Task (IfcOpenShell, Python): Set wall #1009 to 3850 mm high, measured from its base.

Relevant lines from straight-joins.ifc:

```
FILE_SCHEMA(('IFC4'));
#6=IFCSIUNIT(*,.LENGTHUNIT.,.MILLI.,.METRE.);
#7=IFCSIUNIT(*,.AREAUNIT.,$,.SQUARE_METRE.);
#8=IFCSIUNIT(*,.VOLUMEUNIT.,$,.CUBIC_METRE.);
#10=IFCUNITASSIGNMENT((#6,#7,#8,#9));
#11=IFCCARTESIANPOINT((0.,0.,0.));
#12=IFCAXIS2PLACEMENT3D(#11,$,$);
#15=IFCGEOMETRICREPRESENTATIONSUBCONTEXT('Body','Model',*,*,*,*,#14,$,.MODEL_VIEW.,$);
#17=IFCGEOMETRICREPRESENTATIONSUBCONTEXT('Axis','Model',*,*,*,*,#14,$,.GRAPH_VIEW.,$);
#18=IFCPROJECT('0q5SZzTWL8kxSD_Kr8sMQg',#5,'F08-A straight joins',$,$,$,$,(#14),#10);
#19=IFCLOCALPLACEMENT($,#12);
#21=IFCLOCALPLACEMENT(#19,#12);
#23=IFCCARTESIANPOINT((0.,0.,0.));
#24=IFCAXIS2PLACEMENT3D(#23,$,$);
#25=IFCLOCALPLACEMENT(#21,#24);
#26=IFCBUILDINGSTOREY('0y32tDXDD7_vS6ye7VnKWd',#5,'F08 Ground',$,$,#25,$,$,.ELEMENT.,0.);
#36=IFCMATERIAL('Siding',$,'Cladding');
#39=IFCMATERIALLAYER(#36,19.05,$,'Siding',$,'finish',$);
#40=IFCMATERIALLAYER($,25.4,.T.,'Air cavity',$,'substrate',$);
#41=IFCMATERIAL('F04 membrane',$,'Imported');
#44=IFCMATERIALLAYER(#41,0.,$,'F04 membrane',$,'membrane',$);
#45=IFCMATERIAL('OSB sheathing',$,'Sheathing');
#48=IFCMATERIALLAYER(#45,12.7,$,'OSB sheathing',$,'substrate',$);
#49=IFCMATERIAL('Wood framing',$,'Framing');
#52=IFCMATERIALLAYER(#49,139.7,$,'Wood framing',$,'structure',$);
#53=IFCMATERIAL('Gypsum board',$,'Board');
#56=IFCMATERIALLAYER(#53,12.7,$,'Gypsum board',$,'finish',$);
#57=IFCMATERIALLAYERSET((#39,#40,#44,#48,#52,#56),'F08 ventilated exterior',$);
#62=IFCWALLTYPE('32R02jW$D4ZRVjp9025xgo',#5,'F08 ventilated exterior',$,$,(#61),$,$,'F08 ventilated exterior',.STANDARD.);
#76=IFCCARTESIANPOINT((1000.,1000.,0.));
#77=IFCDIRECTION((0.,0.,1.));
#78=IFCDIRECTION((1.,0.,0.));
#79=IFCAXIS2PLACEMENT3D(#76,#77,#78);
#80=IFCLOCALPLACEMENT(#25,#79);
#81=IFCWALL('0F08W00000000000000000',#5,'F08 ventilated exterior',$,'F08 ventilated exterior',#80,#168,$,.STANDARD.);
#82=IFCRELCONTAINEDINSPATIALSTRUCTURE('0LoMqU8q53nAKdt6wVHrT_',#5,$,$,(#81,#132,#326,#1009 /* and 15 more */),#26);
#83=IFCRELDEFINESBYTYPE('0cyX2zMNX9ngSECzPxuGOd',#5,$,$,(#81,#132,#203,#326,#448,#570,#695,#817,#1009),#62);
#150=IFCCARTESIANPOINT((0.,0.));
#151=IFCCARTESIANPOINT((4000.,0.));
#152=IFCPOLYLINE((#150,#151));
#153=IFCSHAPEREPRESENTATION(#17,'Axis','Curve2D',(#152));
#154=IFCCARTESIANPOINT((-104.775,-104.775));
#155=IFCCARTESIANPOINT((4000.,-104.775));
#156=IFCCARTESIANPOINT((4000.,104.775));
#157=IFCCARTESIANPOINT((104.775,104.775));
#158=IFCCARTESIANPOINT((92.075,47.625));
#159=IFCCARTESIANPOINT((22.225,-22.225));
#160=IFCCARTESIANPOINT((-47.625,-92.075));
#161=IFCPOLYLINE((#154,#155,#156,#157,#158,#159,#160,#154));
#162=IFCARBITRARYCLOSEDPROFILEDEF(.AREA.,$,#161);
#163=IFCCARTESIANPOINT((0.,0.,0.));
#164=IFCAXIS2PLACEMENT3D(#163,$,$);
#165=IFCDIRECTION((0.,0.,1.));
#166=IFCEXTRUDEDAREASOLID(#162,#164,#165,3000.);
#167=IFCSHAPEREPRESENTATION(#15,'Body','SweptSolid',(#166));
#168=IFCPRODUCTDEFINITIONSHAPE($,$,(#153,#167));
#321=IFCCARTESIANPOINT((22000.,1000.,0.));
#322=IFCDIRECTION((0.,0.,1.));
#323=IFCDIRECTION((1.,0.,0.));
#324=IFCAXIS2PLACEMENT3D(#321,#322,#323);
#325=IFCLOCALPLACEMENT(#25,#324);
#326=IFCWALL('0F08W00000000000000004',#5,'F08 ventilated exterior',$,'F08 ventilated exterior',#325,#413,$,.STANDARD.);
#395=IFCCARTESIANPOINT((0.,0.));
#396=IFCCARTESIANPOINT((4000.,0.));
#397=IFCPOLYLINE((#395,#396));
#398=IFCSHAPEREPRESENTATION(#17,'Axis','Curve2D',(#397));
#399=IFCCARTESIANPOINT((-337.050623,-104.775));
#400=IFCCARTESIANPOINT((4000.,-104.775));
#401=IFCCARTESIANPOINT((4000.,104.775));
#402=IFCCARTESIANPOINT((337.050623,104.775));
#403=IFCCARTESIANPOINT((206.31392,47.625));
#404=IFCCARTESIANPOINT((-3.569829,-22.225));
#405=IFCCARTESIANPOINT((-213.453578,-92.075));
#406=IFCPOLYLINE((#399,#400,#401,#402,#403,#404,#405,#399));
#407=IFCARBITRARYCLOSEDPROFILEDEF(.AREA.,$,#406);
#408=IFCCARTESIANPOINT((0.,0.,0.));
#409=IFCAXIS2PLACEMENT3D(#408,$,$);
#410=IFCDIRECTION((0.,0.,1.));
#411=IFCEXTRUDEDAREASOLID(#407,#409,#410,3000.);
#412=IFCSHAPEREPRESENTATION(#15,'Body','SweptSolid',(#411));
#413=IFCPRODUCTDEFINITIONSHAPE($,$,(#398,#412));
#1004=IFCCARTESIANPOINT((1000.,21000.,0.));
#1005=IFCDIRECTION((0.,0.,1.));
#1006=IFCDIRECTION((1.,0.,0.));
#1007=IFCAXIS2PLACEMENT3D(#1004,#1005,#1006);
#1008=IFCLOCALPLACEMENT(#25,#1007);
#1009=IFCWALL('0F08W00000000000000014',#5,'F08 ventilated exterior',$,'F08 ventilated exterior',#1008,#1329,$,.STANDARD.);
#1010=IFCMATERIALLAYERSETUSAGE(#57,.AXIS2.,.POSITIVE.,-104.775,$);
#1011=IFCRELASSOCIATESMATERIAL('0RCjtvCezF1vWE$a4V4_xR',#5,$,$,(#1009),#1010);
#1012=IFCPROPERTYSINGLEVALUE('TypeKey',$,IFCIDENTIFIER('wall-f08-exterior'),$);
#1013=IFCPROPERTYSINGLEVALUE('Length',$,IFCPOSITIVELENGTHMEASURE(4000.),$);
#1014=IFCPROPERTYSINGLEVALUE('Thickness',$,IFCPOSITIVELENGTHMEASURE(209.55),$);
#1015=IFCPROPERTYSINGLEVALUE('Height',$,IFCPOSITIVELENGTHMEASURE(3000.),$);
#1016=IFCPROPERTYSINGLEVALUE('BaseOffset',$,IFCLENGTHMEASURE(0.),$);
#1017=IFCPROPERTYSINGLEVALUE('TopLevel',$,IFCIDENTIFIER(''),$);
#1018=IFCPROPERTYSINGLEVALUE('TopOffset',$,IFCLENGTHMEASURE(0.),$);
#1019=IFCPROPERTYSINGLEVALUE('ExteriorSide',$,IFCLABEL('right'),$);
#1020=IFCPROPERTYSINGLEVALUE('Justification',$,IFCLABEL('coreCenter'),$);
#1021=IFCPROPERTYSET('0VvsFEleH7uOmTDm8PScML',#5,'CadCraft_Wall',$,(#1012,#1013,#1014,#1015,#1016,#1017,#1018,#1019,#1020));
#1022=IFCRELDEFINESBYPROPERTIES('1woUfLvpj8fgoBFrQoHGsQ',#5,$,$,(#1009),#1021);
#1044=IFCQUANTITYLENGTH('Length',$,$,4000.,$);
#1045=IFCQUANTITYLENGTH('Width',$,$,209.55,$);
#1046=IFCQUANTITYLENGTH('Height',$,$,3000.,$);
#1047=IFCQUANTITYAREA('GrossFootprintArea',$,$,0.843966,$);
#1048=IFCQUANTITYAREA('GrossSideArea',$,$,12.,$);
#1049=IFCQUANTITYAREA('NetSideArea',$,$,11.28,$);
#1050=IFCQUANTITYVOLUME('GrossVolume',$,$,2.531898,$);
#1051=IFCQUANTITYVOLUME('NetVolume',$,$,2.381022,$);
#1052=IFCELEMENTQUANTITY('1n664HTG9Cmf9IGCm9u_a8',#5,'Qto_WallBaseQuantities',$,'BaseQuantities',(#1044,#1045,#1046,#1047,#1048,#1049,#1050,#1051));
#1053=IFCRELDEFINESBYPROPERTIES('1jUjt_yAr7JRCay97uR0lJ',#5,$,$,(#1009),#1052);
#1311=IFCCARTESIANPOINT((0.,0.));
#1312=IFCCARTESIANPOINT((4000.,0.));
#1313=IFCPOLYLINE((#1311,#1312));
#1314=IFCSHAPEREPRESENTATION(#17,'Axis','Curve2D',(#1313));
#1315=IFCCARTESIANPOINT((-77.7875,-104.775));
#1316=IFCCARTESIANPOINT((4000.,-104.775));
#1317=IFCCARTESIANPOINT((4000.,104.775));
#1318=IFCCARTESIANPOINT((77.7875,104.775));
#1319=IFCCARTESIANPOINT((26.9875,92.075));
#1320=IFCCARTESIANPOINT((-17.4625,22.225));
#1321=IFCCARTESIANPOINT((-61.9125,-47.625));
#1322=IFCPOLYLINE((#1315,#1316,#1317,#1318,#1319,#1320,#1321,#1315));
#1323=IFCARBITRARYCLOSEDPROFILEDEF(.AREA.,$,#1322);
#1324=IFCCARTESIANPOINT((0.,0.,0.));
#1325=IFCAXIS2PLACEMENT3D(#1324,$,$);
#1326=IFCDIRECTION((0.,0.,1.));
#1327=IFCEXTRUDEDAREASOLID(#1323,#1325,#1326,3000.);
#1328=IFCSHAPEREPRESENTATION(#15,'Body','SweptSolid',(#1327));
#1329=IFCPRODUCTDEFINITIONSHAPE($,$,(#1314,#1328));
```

```python
import ifcopenshell
import ifcopenshell.api.pset
import ifcopenshell.geom
import ifcopenshell.util.element
import ifcopenshell.util.representation
import ifcopenshell.util.shape
import ifcopenshell.util.unit

model = ifcopenshell.open("straight-joins.ifc")
unit_scale = ifcopenshell.util.unit.calculate_unit_scale(model)
area_scale = ifcopenshell.util.unit.calculate_unit_scale(model, "AREAUNIT")
volume_scale = ifcopenshell.util.unit.calculate_unit_scale(model, "VOLUMEUNIT")
settings = ifcopenshell.geom.settings()


def volume(element):
    """Net volume in cubic metres, openings subtracted."""
    shape = ifcopenshell.geom.create_shape(settings, element)
    return ifcopenshell.util.shape.get_volume(shape.geometry)


wall = model.by_guid("0F08W00000000000000014")
before = volume(wall)

body = ifcopenshell.util.representation.get_representation(wall, "Model", "Body")
solid = body.Items[0]
old_height = solid.Depth
solid.Depth = 3850.0
after = volume(wall)
thickness = 0.2096  # wall thickness in metres

# Update the stored height, areas and volumes.
pset = model.by_id(ifcopenshell.util.element.get_pset(wall, "CadCraft_Wall", should_inherit=False)["id"])
ifcopenshell.api.pset.edit_pset(model, pset=pset, properties={
    "Height": model.create_entity("IfcPositiveLengthMeasure", solid.Depth),
})
qto = model.by_id(ifcopenshell.util.element.get_pset(wall, "Qto_WallBaseQuantities", should_inherit=False)["id"])
ifcopenshell.api.pset.edit_qto(model, qto=qto, properties={
    "Height": solid.Depth,
    "GrossSideArea": ifcopenshell.util.element.get_pset(wall, "Qto_WallBaseQuantities", "GrossSideArea") * solid.Depth / old_height,
    "NetSideArea": after / thickness / area_scale,
    "GrossVolume": ifcopenshell.util.element.get_pset(wall, "Qto_WallBaseQuantities", "GrossVolume") * solid.Depth / old_height,
    "NetVolume": after / volume_scale,
})

print(f"height {old_height:g} -> {solid.Depth:g}, volume {before:.3f} -> {after:.3f} m3")

model.write("straight-joins_updated.ifc")
```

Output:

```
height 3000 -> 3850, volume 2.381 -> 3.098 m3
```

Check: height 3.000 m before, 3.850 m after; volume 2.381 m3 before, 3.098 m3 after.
